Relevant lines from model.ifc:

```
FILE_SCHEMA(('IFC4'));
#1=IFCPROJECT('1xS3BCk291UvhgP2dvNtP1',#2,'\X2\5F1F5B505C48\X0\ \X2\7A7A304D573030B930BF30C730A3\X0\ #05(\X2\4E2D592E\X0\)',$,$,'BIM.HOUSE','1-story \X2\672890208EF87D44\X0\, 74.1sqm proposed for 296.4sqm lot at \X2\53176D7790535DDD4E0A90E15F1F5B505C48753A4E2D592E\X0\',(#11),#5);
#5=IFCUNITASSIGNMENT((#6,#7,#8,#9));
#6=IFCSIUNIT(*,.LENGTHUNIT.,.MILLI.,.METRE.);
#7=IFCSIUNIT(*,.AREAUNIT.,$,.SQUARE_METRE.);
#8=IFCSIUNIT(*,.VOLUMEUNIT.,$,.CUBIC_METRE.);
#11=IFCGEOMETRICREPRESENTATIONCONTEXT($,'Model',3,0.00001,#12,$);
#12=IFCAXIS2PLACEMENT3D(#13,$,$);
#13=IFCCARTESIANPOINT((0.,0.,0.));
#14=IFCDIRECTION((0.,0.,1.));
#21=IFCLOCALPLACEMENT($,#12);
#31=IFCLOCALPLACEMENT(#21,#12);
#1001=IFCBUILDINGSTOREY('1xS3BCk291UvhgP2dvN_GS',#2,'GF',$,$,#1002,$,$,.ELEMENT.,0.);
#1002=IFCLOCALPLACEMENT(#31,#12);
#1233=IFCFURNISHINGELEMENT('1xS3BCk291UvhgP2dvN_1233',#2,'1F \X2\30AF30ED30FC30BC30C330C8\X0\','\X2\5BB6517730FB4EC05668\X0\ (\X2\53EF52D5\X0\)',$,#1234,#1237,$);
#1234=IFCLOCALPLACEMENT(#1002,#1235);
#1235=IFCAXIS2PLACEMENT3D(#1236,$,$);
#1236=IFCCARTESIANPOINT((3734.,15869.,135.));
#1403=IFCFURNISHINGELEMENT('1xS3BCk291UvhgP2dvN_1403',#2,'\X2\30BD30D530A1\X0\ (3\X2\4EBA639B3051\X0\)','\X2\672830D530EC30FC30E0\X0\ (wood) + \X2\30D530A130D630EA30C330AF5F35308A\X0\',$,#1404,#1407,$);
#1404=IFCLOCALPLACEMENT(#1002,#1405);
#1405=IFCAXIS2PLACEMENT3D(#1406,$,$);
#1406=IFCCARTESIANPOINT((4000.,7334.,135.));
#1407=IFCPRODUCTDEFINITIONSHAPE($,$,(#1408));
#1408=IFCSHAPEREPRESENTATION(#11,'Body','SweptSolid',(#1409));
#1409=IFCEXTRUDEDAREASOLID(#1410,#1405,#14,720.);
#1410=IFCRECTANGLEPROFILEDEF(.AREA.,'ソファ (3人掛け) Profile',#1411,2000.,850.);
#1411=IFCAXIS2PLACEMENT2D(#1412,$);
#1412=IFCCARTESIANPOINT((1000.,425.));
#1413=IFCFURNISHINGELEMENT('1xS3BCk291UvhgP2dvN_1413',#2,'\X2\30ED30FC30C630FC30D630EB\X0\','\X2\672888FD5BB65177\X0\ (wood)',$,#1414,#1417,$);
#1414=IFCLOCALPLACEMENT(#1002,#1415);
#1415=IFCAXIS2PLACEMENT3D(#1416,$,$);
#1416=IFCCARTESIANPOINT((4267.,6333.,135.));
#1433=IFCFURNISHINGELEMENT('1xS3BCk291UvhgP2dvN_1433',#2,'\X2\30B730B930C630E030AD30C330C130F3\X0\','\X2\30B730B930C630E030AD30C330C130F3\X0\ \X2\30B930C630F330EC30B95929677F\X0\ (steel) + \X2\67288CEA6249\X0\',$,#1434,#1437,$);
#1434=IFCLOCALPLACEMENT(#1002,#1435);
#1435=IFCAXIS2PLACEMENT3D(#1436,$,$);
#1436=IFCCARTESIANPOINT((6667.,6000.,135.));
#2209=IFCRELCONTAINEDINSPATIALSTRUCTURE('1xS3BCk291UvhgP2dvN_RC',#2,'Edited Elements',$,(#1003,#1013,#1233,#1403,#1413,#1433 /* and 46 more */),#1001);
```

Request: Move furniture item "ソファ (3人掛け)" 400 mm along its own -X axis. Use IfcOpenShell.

```python
import ifcopenshell
import ifcopenshell.api.geometry
import ifcopenshell.util.placement

model = ifcopenshell.open("model.ifc")

item = model.by_guid("1xS3BCk291UvhgP2dvN_1403")
matrix = ifcopenshell.util.placement.get_local_placement(item.ObjectPlacement)
matrix[:3, 3] -= matrix[:3, 0] * 400.0
ifcopenshell.api.geometry.edit_object_placement(model, product=item, matrix=matrix, is_si=False)

print(ifcopenshell.util.placement.get_local_placement(item.ObjectPlacement).round(3) + 0.0)

model.write("model_edited.ifc")
```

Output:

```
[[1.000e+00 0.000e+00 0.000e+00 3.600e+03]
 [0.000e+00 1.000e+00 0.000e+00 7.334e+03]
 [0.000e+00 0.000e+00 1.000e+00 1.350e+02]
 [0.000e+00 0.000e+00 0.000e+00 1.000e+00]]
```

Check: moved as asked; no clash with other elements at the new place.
